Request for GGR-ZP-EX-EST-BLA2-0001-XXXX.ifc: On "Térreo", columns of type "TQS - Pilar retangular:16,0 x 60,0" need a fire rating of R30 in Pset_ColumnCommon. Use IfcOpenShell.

First a look at what the model holds.

```python
import ifcopenshell
import ifcopenshell.util.element

model = ifcopenshell.open("GGR-ZP-EX-EST-BLA2-0001-XXXX.ifc")
print(model.schema)
storey = next(s for s in model.by_type("IfcBuildingStorey") if s.Name == "Térreo")
columns = [e for e in ifcopenshell.util.element.get_decomposition(storey) if e.is_a("IfcColumn")]
seen = {}
for e in columns:
    element_type = ifcopenshell.util.element.get_type(e)
    key = (element_type.Name if element_type != e and element_type else None, ifcopenshell.util.element.get_pset(e, "Pset_ColumnCommon", "FireRating"))
    seen[key] = seen.get(key, 0) + 1
for (name, value), count in sorted(seen.items(), key=str):
    print(count, "x", name, "|", value)
```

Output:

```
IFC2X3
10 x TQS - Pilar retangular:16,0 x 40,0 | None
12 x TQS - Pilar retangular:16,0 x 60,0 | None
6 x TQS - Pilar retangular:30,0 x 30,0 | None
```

```python
import ifcopenshell
import ifcopenshell.api.pset
import ifcopenshell.util.element

model = ifcopenshell.open("GGR-ZP-EX-EST-BLA2-0001-XXXX.ifc")

storey = next(s for s in model.by_type("IfcBuildingStorey") if s.Name == "Térreo")
columns = [e for e in ifcopenshell.util.element.get_decomposition(storey) if e.is_a("IfcColumn")]

count = 0
for e in columns:
    element_type = ifcopenshell.util.element.get_type(e)
    if element_type in (None, e) or element_type.Name != "TQS - Pilar retangular:16,0 x 60,0":
        continue
    # add_pset returns the element's existing set when there is one.
    pset = ifcopenshell.api.pset.add_pset(model, product=e, name="Pset_ColumnCommon")
    ifcopenshell.api.pset.edit_pset(model, pset=pset, properties={"FireRating": "R30"})
    count += 1

print(count, "columns updated")

model.write("GGR-ZP-EX-EST-BLA2-0001-XXXX_edited.ifc")
```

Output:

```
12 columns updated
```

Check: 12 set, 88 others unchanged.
